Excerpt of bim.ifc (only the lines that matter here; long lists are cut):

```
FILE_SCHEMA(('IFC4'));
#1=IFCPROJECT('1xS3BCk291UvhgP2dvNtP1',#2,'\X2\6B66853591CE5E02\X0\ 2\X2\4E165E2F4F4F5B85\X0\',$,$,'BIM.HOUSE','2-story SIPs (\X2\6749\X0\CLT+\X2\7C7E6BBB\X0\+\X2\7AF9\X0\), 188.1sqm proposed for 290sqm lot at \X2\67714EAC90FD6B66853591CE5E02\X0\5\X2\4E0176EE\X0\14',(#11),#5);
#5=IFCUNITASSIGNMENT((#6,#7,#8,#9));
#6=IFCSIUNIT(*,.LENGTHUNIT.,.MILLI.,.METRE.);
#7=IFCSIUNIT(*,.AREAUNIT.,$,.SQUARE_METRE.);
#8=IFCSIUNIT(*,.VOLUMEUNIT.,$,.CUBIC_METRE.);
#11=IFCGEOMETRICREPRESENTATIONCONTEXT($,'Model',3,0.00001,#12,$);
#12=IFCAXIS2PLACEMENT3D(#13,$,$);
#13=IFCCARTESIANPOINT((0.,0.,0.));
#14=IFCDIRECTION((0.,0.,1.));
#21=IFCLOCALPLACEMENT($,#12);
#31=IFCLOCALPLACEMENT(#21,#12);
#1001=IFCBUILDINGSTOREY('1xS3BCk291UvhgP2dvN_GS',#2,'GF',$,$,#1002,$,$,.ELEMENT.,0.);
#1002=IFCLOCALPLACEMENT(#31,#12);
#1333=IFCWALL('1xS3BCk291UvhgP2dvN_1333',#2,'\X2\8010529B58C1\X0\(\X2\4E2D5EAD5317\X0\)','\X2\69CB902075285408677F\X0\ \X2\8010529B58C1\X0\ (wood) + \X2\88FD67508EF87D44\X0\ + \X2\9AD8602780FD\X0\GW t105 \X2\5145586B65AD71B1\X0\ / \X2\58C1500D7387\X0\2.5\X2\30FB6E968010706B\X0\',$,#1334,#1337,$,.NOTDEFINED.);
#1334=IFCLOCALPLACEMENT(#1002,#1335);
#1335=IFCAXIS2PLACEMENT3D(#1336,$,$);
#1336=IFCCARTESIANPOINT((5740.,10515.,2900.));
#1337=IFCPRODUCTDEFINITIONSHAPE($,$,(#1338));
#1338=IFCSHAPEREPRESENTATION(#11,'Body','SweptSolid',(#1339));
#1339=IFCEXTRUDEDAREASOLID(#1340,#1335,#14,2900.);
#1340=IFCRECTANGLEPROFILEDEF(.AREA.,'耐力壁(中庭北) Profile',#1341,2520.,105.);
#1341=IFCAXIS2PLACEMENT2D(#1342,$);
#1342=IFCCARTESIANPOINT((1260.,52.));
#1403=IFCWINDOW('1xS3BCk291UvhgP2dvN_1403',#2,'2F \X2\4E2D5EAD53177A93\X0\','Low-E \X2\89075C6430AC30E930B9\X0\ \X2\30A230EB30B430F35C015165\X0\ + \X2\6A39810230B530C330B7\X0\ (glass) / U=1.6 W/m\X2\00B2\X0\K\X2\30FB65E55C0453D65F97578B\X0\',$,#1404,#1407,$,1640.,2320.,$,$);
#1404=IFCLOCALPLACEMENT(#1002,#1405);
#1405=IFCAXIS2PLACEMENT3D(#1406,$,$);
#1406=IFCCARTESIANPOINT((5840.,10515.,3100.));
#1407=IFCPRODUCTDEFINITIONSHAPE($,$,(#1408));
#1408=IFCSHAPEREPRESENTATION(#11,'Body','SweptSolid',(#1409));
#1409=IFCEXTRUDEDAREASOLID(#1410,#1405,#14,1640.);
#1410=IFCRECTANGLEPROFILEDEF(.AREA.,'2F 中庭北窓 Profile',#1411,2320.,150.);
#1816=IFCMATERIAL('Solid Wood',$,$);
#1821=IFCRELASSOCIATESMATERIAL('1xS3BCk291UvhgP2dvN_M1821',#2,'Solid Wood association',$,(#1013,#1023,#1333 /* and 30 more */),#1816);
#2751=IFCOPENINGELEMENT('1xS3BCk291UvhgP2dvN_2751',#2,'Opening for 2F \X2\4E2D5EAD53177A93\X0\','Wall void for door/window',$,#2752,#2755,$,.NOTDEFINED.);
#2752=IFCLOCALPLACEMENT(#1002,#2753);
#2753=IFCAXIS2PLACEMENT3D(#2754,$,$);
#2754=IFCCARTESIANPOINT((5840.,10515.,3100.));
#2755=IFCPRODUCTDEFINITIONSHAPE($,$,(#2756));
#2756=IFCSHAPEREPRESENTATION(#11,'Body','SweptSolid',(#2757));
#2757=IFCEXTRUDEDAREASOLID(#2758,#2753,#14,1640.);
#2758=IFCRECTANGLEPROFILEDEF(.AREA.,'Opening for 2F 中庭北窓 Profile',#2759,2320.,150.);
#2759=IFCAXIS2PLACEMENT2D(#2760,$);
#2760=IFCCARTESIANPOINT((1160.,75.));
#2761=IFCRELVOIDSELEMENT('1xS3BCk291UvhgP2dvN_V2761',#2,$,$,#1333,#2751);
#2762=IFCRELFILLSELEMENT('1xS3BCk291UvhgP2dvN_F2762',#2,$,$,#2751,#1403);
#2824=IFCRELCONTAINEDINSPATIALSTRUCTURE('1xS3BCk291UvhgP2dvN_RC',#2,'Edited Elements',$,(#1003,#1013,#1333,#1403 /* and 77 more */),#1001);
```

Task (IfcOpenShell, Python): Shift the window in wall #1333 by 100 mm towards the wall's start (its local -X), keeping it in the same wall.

```python
import ifcopenshell
import ifcopenshell.api.geometry
import ifcopenshell.util.placement
import ifcopenshell.util.unit

model = ifcopenshell.open("bim.ifc")
unit_scale = ifcopenshell.util.unit.calculate_unit_scale(model)

window = model.by_guid("1xS3BCk291UvhgP2dvN_1403")
opening = window.FillsVoids[0].RelatingOpeningElement
wall = opening.VoidsElements[0].RelatingBuildingElement

wall_matrix = ifcopenshell.util.placement.get_local_placement(wall.ObjectPlacement)
shift = wall_matrix[:3, 0] * -0.1 / unit_scale
before = ifcopenshell.util.placement.get_local_placement(window.ObjectPlacement)[:3, 3].copy()

# The window is not placed relative to its opening, so move both.
for product in (opening, window):
    matrix = ifcopenshell.util.placement.get_local_placement(product.ObjectPlacement)
    matrix[:3, 3] += shift
    ifcopenshell.api.geometry.edit_object_placement(model, product=product, matrix=matrix, is_si=False)

after = ifcopenshell.util.placement.get_local_placement(window.ObjectPlacement)[:3, 3]
print("window moved by", (after - before).round(3) + 0.0)

model.write("bim_v2.ifc")
```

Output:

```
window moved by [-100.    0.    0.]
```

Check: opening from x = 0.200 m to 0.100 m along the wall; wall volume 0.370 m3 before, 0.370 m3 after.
